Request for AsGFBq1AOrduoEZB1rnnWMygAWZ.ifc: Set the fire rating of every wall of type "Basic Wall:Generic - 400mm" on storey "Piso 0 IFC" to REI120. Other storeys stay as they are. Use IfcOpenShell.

First a look at what the model holds.

```python
import ifcopenshell
import ifcopenshell.util.element

model = ifcopenshell.open("AsGFBq1AOrduoEZB1rnnWMygAWZ.ifc")
print(model.schema)
storey = next(s for s in model.by_type("IfcBuildingStorey") if s.Name == "Piso 0 IFC")
walls = [e for e in ifcopenshell.util.element.get_decomposition(storey) if e.is_a("IfcWall")]
seen = {}
for e in walls:
    element_type = ifcopenshell.util.element.get_type(e)
    key = (element_type.Name if element_type != e and element_type else None, ifcopenshell.util.element.get_pset(e, "Pset_WallCommon", "FireRating"))
    seen[key] = seen.get(key, 0) + 1
for (name, value), count in sorted(seen.items(), key=str):
    print(count, "x", name, "|", value)
```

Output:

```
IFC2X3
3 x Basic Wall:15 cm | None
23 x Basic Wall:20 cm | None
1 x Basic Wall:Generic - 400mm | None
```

```python
import ifcopenshell
import ifcopenshell.api.pset
import ifcopenshell.util.element

model = ifcopenshell.open("AsGFBq1AOrduoEZB1rnnWMygAWZ.ifc")

storey = next(s for s in model.by_type("IfcBuildingStorey") if s.Name == "Piso 0 IFC")
walls = [e for e in ifcopenshell.util.element.get_decomposition(storey) if e.is_a("IfcWall")]

count = 0
for e in walls:
    element_type = ifcopenshell.util.element.get_type(e)
    if element_type in (None, e) or element_type.Name != "Basic Wall:Generic - 400mm":
        continue
    # add_pset returns the element's existing set when there is one.
    pset = ifcopenshell.api.pset.add_pset(model, product=e, name="Pset_WallCommon")
    ifcopenshell.api.pset.edit_pset(model, pset=pset, properties={"FireRating": "REI120"})
    count += 1

print(count, "walls updated")

model.write("AsGFBq1AOrduoEZB1rnnWMygAWZ_updated.ifc")
```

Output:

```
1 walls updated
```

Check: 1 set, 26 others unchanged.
